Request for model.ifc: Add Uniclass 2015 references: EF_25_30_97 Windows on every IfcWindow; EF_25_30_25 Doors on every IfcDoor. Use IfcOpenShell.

First a look at what the model holds.

```python
import ifcopenshell

model = ifcopenshell.open("model.ifc")
print(model.schema)
print("classifications:", [c.Name for c in model.by_type("IfcClassification")])
for ifc_class in ("IfcDoor", "IfcRoof", "IfcStair", "IfcWall", "IfcWindow"):
    print(ifc_class, len(model.by_type(ifc_class)))
```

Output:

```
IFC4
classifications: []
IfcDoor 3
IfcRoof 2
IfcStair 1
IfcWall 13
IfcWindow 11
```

```python
import ifcopenshell
import ifcopenshell.api.classification

model = ifcopenshell.open("model.ifc")

system = ifcopenshell.api.classification.add_classification(model, classification="Uniclass 2015")

codes = {
    "IfcWindow": ("EF_25_30_97", "Windows"),
    "IfcDoor": ("EF_25_30_25", "Doors"),
}
for ifc_class, (code, name) in codes.items():
    products = model.by_type(ifc_class)
    ifcopenshell.api.classification.add_reference(
        model, products=products, classification=system, identification=code, name=name
    )
    print(code, len(products))

model.write("model_edited.ifc")
```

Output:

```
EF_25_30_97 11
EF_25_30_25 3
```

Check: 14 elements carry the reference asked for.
